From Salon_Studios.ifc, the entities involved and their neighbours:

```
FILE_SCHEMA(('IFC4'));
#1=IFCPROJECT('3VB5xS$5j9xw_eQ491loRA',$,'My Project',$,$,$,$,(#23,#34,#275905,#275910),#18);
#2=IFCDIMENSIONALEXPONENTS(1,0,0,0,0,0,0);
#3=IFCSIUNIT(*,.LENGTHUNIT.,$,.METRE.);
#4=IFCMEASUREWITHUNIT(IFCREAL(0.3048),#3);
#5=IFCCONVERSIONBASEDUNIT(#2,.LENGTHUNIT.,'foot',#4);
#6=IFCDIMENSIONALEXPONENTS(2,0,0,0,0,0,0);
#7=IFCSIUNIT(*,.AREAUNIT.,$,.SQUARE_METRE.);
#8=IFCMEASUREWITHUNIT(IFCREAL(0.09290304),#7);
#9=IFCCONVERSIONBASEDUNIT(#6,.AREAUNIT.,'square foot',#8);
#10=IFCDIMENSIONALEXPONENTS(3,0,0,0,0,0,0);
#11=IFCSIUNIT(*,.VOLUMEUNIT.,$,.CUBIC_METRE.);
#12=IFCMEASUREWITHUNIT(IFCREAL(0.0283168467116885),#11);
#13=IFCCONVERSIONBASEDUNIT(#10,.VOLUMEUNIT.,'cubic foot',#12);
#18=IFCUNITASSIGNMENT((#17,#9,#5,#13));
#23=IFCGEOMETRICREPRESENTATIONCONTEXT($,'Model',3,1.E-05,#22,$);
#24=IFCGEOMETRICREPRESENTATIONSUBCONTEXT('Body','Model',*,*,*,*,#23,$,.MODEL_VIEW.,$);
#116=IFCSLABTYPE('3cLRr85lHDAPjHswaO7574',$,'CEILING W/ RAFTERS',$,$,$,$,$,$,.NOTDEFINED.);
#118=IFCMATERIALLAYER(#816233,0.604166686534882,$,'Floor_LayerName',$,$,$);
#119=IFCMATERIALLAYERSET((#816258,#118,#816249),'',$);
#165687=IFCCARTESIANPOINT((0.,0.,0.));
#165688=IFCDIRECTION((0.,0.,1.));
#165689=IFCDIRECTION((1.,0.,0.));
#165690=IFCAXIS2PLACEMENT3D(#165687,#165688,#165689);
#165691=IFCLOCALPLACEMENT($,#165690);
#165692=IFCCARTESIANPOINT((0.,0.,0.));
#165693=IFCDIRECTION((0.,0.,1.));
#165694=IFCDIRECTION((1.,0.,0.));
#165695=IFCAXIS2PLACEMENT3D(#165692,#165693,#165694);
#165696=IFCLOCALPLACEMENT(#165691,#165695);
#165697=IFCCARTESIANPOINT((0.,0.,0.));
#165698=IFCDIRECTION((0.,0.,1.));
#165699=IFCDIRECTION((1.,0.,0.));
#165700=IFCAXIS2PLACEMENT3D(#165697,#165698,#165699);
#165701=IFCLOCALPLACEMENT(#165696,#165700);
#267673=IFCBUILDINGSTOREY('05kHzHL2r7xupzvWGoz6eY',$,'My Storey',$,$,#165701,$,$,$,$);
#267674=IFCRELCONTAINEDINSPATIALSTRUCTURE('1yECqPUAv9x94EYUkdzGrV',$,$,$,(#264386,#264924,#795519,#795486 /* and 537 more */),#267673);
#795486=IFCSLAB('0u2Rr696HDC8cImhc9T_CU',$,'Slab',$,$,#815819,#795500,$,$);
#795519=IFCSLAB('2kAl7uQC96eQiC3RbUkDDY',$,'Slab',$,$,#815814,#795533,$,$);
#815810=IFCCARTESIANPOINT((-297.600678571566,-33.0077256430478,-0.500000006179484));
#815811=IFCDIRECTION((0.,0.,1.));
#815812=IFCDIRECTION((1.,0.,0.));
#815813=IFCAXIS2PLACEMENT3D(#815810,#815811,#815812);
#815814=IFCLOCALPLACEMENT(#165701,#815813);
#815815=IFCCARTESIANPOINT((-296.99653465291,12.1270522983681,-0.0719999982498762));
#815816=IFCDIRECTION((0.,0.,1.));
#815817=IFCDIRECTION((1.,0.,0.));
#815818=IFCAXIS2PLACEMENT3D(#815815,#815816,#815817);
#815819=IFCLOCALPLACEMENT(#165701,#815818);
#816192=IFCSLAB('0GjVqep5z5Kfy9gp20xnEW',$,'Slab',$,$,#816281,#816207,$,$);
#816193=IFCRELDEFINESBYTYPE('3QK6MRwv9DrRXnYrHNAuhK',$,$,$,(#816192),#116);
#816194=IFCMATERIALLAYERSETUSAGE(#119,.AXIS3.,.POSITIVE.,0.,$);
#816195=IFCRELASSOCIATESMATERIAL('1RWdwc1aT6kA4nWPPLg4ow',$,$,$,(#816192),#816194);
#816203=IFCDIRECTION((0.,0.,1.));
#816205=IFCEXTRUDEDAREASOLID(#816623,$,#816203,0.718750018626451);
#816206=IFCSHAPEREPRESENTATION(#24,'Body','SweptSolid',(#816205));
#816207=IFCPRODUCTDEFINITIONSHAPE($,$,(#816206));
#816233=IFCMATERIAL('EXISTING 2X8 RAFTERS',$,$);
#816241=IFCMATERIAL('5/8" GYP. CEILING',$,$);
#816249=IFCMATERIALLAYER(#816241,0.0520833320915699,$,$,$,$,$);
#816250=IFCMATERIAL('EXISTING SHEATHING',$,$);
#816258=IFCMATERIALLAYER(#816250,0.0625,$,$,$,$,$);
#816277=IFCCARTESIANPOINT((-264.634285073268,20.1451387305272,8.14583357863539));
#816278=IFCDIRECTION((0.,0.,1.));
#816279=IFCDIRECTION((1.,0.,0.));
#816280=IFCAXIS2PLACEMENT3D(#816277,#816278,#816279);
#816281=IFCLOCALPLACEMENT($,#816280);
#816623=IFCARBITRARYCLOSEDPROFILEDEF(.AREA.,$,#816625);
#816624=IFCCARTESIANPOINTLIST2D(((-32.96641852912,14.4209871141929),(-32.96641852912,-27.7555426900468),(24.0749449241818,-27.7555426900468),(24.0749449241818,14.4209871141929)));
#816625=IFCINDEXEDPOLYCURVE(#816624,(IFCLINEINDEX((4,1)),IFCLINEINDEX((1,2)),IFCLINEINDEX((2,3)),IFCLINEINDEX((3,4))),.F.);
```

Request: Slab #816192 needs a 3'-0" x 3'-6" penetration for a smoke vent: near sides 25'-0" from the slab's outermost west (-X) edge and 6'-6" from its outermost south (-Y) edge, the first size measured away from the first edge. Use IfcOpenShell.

```python
import numpy as np
import ifcopenshell
import ifcopenshell.api.feature
import ifcopenshell.api.geometry
import ifcopenshell.api.root
import ifcopenshell.geom
import ifcopenshell.util.placement
import ifcopenshell.util.representation
import ifcopenshell.util.shape
import ifcopenshell.util.unit

model = ifcopenshell.open("Salon_Studios.ifc")
unit_scale = ifcopenshell.util.unit.calculate_unit_scale(model)
settings = ifcopenshell.geom.settings()


def volume(element):
    """Net volume in cubic metres, openings subtracted."""
    shape = ifcopenshell.geom.create_shape(settings, element)
    return ifcopenshell.util.shape.get_volume(shape.geometry)


slab = model.by_guid("0GjVqep5z5Kfy9gp20xnEW")
before = volume(slab)

# Extent in the slab's own axes, in metres. The edges named are its -X and -Y sides.
slab_shape = ifcopenshell.geom.create_shape(settings, slab)
vertices = ifcopenshell.util.shape.get_vertices(slab_shape.geometry)
x_min, y_min, bottom = vertices.min(axis=0)
top = vertices[:, 2].max()

opening = ifcopenshell.api.root.create_entity(model, ifc_class="IfcOpeningElement", name="Smoke vent opening", predefined_type="OPENING")
context = ifcopenshell.util.representation.get_context(model, "Model", "Body", "MODEL_VIEW")
width, depth = 0.9144, 1.0668
outline = [(0.0, 0.0), (width, 0.0), (width, depth), (0.0, depth), (0.0, 0.0)]
# Overshoot both faces by 50 mm so the cut is clean.
shape = ifcopenshell.api.geometry.add_slab_representation(
    model, context=context, depth=top - bottom + 0.1, polyline=outline
)
ifcopenshell.api.geometry.assign_representation(model, product=opening, representation=shape)

matrix = ifcopenshell.util.placement.get_local_placement(slab.ObjectPlacement)
matrix[:, 3] = matrix @ np.append(np.array([x_min + 7.62, y_min + 1.9812, bottom - 0.05]) / unit_scale, 1.0)
ifcopenshell.api.geometry.edit_object_placement(model, product=opening, matrix=matrix, is_si=False)
ifcopenshell.api.feature.add_feature(model, feature=opening, element=slab)

after = volume(slab)

print(f"slab volume {before:.3f} -> {after:.3f} m3")

model.write("Salon_Studios_v2.ifc")
```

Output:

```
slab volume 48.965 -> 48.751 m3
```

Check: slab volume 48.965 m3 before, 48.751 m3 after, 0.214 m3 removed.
